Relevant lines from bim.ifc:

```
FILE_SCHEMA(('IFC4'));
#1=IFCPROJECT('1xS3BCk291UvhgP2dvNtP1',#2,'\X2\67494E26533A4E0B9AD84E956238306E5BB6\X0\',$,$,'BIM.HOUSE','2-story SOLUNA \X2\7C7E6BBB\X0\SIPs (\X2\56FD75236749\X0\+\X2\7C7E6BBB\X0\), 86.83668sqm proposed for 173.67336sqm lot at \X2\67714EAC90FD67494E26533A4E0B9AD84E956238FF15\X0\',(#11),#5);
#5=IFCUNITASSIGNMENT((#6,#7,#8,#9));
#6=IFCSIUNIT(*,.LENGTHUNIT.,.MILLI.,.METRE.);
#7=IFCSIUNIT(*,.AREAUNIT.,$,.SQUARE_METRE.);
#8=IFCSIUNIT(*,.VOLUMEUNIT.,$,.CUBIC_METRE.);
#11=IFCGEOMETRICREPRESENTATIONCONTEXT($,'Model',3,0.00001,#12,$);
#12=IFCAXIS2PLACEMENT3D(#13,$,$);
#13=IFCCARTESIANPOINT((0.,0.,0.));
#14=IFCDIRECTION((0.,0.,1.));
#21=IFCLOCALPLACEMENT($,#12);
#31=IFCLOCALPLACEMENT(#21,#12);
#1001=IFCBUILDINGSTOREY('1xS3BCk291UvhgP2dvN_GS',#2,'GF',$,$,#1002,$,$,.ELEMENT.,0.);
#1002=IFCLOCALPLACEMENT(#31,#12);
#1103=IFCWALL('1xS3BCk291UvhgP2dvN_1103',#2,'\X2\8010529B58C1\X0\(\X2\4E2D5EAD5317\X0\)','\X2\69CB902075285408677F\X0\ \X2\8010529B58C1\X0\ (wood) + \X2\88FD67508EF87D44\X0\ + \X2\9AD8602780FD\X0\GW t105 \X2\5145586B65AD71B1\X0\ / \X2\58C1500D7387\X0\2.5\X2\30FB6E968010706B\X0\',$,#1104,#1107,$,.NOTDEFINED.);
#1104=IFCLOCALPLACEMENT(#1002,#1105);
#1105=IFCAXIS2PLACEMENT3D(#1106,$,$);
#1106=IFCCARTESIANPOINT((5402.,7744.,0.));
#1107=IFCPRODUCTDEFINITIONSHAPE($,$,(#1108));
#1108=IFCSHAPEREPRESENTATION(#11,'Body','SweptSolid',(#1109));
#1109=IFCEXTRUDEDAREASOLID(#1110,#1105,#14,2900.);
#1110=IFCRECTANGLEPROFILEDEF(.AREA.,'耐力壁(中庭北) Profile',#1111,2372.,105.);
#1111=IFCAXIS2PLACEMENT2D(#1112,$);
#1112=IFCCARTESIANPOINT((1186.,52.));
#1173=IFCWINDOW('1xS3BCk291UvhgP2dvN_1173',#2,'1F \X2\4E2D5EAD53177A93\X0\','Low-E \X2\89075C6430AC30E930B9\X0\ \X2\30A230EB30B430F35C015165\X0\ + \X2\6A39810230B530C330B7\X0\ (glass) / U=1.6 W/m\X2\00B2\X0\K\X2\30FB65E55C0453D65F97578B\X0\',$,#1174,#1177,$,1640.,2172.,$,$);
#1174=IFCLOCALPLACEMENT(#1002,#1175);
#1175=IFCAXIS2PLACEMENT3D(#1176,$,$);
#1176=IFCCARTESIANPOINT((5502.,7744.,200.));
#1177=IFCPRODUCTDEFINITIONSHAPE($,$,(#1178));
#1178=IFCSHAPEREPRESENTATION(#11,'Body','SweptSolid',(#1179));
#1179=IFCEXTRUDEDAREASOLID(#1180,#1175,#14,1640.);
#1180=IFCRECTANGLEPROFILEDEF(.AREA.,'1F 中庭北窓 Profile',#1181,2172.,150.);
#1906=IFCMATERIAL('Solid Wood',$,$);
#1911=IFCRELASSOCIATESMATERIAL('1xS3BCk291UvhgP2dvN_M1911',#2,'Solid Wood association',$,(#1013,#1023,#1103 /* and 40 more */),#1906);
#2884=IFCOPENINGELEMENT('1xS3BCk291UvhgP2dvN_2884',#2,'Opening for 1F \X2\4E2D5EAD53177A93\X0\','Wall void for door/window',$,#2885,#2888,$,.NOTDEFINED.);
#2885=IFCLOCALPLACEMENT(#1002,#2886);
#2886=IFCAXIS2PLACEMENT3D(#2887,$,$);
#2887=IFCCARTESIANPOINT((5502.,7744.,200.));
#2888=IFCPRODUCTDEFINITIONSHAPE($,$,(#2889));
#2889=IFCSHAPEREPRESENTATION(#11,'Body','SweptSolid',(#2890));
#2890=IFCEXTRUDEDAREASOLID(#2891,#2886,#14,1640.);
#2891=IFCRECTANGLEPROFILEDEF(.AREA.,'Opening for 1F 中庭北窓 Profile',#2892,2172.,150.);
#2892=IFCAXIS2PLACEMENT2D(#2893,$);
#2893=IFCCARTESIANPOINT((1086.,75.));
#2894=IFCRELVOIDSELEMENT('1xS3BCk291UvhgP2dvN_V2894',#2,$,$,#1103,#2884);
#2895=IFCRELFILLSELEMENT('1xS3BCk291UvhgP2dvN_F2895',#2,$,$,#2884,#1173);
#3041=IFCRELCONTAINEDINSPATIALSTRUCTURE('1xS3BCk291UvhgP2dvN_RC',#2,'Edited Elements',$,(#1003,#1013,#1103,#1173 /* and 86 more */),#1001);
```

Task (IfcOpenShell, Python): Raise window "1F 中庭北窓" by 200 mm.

```python
import numpy as np
import ifcopenshell
import ifcopenshell.api.geometry
import ifcopenshell.util.placement
import ifcopenshell.util.unit

model = ifcopenshell.open("bim.ifc")
unit_scale = ifcopenshell.util.unit.calculate_unit_scale(model)

window = model.by_guid("1xS3BCk291UvhgP2dvN_1173")
opening = window.FillsVoids[0].RelatingOpeningElement
dz = 0.2 / unit_scale

shift = np.array([0.0, 0.0, dz])
# The window is not placed relative to its opening, so move both.
for product in (opening, window):
    matrix = ifcopenshell.util.placement.get_local_placement(product.ObjectPlacement)
    matrix[:3, 3] += shift
    ifcopenshell.api.geometry.edit_object_placement(model, product=product, matrix=matrix, is_si=False)

print(f"moved by {dz * unit_scale:+.3f} m")

model.write("bim_rev.ifc")
```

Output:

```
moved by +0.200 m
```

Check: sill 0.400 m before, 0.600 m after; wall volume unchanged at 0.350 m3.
